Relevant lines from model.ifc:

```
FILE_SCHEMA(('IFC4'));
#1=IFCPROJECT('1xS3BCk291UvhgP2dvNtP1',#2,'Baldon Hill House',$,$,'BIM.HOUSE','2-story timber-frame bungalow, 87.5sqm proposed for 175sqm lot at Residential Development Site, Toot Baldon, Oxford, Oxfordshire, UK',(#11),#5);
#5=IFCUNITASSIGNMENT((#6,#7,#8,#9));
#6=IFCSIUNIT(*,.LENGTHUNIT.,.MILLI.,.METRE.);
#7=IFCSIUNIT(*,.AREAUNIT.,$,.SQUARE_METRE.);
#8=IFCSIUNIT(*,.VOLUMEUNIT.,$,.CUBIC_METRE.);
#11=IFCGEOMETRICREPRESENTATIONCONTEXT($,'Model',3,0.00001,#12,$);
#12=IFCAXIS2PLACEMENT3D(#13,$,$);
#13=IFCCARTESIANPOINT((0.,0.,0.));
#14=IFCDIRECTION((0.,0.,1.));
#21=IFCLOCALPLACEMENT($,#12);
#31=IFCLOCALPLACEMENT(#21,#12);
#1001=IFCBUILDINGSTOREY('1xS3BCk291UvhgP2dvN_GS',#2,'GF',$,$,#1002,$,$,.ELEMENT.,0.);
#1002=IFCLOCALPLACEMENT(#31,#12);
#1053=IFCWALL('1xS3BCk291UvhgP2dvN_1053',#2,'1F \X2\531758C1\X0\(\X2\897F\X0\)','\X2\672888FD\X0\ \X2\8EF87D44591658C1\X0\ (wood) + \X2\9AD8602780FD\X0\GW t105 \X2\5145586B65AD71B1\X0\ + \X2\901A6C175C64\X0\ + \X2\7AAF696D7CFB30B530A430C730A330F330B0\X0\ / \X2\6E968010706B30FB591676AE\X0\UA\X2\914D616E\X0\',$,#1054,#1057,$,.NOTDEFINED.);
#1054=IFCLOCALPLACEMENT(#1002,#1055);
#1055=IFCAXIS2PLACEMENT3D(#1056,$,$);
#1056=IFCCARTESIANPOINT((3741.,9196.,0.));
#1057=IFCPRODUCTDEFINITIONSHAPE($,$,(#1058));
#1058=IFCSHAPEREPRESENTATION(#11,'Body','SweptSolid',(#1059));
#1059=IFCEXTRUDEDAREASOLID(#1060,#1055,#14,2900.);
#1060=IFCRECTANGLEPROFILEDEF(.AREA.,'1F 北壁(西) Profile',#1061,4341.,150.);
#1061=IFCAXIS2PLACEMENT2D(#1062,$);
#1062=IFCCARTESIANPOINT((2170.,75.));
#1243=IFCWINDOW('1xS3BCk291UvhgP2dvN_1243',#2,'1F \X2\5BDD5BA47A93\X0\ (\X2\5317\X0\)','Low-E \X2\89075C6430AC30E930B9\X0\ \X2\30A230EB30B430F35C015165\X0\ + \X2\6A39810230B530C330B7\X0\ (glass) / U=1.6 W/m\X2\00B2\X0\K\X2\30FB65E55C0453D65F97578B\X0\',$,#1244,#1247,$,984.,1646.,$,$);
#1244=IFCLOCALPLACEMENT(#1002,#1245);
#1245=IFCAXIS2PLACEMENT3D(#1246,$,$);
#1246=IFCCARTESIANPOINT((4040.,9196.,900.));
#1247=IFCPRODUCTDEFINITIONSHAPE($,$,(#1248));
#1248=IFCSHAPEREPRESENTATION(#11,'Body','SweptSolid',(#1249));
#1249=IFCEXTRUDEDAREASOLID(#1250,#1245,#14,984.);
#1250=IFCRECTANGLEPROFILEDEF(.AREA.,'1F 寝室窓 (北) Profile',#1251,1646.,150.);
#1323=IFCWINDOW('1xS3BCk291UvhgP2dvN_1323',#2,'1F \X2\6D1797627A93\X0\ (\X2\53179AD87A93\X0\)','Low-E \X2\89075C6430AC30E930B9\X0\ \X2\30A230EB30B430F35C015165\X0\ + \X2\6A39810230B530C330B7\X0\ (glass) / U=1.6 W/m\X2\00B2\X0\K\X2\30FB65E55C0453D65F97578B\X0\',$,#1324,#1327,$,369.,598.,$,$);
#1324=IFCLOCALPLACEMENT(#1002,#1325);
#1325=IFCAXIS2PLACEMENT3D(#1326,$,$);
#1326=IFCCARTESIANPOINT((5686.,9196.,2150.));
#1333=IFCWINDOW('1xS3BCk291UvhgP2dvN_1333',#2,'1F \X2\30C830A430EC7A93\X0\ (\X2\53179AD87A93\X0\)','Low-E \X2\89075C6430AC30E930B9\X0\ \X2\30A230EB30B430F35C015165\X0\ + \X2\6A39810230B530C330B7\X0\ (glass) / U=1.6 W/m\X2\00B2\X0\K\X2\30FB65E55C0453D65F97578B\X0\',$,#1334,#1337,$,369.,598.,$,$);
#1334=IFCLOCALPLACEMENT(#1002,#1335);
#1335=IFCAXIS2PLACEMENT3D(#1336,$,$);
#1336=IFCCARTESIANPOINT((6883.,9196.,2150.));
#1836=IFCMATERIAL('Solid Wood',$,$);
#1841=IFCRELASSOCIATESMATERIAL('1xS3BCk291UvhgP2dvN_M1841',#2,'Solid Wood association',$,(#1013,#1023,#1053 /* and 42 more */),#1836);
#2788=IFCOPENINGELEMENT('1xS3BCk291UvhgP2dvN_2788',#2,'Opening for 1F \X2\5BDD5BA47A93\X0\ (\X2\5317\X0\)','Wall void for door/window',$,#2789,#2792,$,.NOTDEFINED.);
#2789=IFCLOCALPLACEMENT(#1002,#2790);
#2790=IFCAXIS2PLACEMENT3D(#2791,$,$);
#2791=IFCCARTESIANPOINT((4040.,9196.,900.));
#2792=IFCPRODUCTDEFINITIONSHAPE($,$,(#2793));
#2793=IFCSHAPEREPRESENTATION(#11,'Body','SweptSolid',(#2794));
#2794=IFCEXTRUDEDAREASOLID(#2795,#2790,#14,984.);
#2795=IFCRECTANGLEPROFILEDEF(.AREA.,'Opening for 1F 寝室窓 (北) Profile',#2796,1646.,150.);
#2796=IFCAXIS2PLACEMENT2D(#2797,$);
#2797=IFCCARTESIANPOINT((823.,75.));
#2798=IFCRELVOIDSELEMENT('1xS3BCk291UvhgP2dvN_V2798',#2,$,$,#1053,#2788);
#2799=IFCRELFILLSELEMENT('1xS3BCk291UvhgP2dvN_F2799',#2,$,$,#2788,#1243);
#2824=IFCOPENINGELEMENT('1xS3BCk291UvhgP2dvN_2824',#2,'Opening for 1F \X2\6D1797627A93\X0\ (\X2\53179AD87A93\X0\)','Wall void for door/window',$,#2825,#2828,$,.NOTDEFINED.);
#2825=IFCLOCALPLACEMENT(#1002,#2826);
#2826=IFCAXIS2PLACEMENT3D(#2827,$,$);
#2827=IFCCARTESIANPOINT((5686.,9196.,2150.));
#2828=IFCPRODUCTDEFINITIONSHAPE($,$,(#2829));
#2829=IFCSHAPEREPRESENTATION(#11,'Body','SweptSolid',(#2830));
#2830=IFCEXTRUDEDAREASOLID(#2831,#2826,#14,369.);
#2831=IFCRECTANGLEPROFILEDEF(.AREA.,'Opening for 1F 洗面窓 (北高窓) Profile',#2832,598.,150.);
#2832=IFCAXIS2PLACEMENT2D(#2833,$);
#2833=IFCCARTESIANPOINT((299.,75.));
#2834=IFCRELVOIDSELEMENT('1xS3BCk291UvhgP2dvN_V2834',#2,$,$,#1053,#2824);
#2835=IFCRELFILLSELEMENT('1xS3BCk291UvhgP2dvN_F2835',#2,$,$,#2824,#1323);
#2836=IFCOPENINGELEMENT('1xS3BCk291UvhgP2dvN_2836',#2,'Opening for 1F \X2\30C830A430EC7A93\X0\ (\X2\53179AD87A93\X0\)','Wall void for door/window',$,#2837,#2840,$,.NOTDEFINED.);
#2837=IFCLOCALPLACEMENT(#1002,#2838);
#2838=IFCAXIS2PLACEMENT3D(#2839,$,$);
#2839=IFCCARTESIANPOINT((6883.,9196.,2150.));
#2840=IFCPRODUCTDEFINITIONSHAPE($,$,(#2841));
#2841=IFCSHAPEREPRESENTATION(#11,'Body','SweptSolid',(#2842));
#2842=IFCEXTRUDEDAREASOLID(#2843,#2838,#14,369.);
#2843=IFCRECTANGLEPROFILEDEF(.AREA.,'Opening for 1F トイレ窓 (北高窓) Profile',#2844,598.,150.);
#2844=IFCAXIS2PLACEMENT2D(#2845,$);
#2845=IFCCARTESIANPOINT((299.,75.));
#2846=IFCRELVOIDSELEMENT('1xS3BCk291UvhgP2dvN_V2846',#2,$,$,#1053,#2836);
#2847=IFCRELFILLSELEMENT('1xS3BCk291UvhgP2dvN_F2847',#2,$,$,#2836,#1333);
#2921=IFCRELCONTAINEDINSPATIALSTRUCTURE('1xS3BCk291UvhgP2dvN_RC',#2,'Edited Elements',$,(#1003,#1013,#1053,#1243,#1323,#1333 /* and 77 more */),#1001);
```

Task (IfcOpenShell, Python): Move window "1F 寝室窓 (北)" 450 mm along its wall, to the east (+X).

```python
import ifcopenshell
import ifcopenshell.api.geometry
import ifcopenshell.util.placement
import ifcopenshell.util.unit

model = ifcopenshell.open("model.ifc")
unit_scale = ifcopenshell.util.unit.calculate_unit_scale(model)

window = model.by_id(1243)
opening = window.FillsVoids[0].RelatingOpeningElement
wall = opening.VoidsElements[0].RelatingBuildingElement

wall_matrix = ifcopenshell.util.placement.get_local_placement(wall.ObjectPlacement)
shift = wall_matrix[:3, 0] * 0.45 / unit_scale
before = ifcopenshell.util.placement.get_local_placement(window.ObjectPlacement)[:3, 3].copy()

# The window is not placed relative to its opening, so move both.
for product in (opening, window):
    matrix = ifcopenshell.util.placement.get_local_placement(product.ObjectPlacement)
    matrix[:3, 3] += shift
    ifcopenshell.api.geometry.edit_object_placement(model, product=product, matrix=matrix, is_si=False)

after = ifcopenshell.util.placement.get_local_placement(window.ObjectPlacement)[:3, 3]
print("window moved by", (after - before).round(3) + 0.0)

model.write("model_v2.ifc")
```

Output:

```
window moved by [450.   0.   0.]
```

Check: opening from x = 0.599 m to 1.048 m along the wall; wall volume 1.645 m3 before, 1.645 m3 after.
